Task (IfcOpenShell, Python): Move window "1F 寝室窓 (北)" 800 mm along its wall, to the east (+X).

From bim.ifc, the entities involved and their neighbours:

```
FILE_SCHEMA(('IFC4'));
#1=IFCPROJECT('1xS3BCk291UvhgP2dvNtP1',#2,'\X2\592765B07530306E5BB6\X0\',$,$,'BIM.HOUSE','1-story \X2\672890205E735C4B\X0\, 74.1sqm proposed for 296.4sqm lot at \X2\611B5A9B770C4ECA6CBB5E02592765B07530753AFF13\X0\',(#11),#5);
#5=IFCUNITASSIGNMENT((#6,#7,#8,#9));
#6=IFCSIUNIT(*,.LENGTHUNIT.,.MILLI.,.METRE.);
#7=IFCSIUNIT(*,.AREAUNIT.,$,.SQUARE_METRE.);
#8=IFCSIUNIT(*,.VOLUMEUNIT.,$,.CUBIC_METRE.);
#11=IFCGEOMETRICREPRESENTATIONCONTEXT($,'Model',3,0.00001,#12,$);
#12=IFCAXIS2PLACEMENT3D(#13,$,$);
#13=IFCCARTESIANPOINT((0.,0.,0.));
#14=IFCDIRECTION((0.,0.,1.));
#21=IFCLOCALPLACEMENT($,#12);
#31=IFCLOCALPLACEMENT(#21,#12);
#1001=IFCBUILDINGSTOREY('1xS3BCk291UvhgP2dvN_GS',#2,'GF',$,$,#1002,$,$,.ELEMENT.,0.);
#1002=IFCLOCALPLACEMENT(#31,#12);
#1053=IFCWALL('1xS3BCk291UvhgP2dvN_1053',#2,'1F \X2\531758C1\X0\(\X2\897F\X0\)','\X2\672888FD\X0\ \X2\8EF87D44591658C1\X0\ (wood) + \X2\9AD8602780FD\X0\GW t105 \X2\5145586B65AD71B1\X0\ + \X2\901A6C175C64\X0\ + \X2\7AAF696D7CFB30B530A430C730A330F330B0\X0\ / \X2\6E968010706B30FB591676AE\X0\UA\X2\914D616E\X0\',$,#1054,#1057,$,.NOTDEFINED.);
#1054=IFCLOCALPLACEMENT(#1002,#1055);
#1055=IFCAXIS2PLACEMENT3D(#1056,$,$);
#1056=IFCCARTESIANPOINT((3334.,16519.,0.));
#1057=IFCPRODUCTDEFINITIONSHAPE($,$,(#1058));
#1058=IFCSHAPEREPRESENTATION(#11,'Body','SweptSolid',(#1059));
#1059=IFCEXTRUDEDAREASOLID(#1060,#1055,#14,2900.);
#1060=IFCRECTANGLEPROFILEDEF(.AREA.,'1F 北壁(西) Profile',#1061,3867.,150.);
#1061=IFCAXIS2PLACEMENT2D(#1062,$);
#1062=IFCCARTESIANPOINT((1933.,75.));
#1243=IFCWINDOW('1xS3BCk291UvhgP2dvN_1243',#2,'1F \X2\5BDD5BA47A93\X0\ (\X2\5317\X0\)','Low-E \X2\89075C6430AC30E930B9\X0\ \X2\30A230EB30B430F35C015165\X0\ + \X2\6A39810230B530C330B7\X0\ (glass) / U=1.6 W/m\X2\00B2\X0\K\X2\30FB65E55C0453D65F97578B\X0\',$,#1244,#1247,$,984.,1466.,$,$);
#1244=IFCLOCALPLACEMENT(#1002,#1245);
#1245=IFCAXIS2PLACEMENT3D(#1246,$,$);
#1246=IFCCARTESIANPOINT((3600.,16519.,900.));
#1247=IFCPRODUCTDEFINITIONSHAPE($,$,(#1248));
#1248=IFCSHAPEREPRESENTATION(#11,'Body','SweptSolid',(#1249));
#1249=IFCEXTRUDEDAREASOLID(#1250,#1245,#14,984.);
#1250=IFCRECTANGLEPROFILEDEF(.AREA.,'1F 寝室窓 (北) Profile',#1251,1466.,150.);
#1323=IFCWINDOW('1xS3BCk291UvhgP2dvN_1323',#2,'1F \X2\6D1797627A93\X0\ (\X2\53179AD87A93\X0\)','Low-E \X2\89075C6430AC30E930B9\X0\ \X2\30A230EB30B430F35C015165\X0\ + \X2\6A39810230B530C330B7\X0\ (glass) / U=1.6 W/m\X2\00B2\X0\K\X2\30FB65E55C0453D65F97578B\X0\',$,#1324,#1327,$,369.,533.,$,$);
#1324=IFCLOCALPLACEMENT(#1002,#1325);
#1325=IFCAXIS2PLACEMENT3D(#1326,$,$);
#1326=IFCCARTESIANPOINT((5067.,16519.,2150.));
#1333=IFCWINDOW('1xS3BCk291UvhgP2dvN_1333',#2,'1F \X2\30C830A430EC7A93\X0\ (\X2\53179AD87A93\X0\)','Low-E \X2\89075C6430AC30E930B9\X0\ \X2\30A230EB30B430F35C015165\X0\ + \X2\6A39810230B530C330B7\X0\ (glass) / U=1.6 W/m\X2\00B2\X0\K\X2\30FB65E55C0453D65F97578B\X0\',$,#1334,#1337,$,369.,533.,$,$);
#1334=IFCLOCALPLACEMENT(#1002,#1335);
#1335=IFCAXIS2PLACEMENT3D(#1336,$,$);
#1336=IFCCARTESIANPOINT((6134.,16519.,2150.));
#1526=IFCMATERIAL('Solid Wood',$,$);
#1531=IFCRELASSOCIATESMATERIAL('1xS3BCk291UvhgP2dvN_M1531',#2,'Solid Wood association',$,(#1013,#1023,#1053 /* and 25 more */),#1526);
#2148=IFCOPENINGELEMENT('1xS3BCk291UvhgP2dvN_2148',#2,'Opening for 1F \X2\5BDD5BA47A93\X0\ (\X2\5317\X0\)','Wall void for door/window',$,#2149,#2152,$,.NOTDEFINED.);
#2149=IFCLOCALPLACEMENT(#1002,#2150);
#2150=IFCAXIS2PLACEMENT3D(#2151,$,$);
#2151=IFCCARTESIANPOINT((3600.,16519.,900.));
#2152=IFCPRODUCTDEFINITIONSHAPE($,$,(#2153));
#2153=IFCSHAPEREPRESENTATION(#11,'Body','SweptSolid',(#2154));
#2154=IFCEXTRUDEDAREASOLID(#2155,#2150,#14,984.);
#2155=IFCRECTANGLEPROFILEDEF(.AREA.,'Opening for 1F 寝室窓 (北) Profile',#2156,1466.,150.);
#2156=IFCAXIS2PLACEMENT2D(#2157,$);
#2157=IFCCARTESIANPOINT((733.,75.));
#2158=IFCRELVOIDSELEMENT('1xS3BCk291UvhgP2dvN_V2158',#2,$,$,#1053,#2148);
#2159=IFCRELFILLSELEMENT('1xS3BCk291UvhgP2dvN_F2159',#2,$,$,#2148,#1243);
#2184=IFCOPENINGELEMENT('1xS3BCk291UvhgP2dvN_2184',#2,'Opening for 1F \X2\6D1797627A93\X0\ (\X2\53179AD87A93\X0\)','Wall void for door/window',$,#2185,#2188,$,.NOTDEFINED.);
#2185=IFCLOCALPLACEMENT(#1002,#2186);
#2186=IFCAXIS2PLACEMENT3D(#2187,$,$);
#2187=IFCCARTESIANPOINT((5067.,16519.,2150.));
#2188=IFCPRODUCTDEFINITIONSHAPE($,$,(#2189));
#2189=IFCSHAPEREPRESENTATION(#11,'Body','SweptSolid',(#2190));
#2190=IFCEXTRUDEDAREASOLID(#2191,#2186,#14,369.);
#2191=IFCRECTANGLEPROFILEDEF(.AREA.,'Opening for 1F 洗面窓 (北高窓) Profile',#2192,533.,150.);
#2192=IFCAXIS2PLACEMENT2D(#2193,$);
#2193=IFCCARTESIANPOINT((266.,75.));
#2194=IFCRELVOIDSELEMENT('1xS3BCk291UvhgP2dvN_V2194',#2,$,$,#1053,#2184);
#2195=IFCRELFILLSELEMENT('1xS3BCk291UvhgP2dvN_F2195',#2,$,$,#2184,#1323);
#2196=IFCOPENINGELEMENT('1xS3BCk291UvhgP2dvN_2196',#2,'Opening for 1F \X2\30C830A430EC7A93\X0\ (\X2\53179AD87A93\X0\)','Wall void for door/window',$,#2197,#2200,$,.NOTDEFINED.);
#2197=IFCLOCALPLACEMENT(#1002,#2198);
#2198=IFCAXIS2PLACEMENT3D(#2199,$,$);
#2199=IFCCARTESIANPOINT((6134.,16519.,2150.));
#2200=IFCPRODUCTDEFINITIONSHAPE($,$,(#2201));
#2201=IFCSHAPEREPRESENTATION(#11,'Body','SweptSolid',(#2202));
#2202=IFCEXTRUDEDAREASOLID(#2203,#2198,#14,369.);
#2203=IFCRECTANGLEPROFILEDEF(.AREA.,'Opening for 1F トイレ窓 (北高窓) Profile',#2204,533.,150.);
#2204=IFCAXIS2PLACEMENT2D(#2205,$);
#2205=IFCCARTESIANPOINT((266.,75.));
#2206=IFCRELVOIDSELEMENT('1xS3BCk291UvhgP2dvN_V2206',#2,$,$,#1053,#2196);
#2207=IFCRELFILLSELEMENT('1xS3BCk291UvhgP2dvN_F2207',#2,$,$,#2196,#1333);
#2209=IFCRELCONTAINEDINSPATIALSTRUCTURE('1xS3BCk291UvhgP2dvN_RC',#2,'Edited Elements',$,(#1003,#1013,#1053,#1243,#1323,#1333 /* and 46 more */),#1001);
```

```python
import ifcopenshell
import ifcopenshell.api.geometry
import ifcopenshell.util.placement
import ifcopenshell.util.unit

model = ifcopenshell.open("bim.ifc")
unit_scale = ifcopenshell.util.unit.calculate_unit_scale(model)

window = model.by_guid("1xS3BCk291UvhgP2dvN_1243")
opening = window.FillsVoids[0].RelatingOpeningElement
wall = opening.VoidsElements[0].RelatingBuildingElement

wall_matrix = ifcopenshell.util.placement.get_local_placement(wall.ObjectPlacement)
shift = wall_matrix[:3, 0] * 0.8 / unit_scale
before = ifcopenshell.util.placement.get_local_placement(window.ObjectPlacement)[:3, 3].copy()

# The window is not placed relative to its opening, so move both.
for product in (opening, window):
    matrix = ifcopenshell.util.placement.get_local_placement(product.ObjectPlacement)
    matrix[:3, 3] += shift
    ifcopenshell.api.geometry.edit_object_placement(model, product=product, matrix=matrix, is_si=False)

after = ifcopenshell.util.placement.get_local_placement(window.ObjectPlacement)[:3, 3]
print("window moved by", (after - before).round(3) + 0.0)

model.write("bim_v2.ifc")
```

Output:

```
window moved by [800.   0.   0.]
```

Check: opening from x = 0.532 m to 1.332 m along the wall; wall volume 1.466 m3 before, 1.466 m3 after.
